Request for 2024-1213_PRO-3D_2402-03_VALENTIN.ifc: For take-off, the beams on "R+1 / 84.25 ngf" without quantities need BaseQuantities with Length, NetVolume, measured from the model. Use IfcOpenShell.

First a look at what the model holds.

```python
import ifcopenshell
import ifcopenshell.util.element
import ifcopenshell.util.unit

model = ifcopenshell.open("2024-1213_PRO-3D_2402-03_VALENTIN.ifc")
print(model.schema)
for unit_type in ("LENGTHUNIT", "AREAUNIT", "VOLUMEUNIT"):
    print(unit_type, ifcopenshell.util.unit.calculate_unit_scale(model, unit_type))
storey = next(s for s in model.by_type("IfcBuildingStorey") if s.Name == "R+1 / 84.25 ngf")
beams = [e for e in ifcopenshell.util.element.get_decomposition(storey) if e.is_a("IfcBeam")]
for e in sorted(beams, key=lambda e: e.id()):
    print(e.id(), e.is_a(), e.Name, list(ifcopenshell.util.element.get_psets(e, qtos_only=True)), sep=" | ")
```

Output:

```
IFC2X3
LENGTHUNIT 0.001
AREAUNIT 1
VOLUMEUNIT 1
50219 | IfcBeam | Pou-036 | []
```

```python
import ifcopenshell
import ifcopenshell.api.pset
import ifcopenshell.geom
import ifcopenshell.util.element
import ifcopenshell.util.shape
import ifcopenshell.util.unit

model = ifcopenshell.open("2024-1213_PRO-3D_2402-03_VALENTIN.ifc")
unit_scale = ifcopenshell.util.unit.calculate_unit_scale(model)
volume_scale = ifcopenshell.util.unit.calculate_unit_scale(model, "VOLUMEUNIT")
settings = ifcopenshell.geom.settings()

storey = next(s for s in model.by_type("IfcBuildingStorey") if s.Name == "R+1 / 84.25 ngf")
beams = [e for e in ifcopenshell.util.element.get_decomposition(storey) if e.is_a("IfcBeam")]

for e in sorted(beams, key=lambda e: e.id()):
    if ifcopenshell.util.element.get_psets(e, qtos_only=True, should_inherit=False):
        continue
    # Geometry comes back in metres, in the element's own axes.
    shape = ifcopenshell.geom.create_shape(settings, e)
    values = {
        "Length": ifcopenshell.util.shape.get_max_xyz(shape.geometry) / unit_scale,
        "NetVolume": ifcopenshell.util.shape.get_volume(shape.geometry) / volume_scale,
    }
    qto = ifcopenshell.api.pset.add_qto(model, product=e, name="BaseQuantities")
    ifcopenshell.api.pset.edit_qto(model, qto=qto, properties=values)
    print(e.id(), {k: round(v, 3) for k, v in values.items()})

model.write("2024-1213_PRO-3D_2402-03_VALENTIN_updated.ifc")
```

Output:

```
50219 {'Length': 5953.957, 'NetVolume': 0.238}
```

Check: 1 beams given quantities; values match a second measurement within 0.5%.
